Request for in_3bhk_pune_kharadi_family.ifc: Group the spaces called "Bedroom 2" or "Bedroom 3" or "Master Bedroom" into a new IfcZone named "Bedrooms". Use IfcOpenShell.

First a look at what the model holds.

```python
import ifcopenshell

model = ifcopenshell.open("in_3bhk_pune_kharadi_family.ifc")
print(model.schema)
seen = {}
for space in model.by_type("IfcSpace"):
    seen[space.LongName] = seen.get(space.LongName, 0) + 1
for name, count in sorted(seen.items(), key=str):
    print(count, "x", name)
print("zones:", [z.Name for z in model.by_type("IfcZone")][:20])
```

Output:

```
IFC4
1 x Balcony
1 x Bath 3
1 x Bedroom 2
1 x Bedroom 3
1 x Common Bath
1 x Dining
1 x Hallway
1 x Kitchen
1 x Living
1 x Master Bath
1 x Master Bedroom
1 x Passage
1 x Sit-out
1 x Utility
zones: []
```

```python
import ifcopenshell
import ifcopenshell.api.group
import ifcopenshell.api.root

model = ifcopenshell.open("in_3bhk_pune_kharadi_family.ifc")

names = {"Bedroom 2", "Bedroom 3", "Master Bedroom"}
spaces = [s for s in model.by_type("IfcSpace") if s.LongName in names]

zone = ifcopenshell.api.root.create_entity(model, ifc_class="IfcZone", name="Bedrooms")
ifcopenshell.api.group.assign_group(model, products=spaces, group=zone)
print(len(spaces), "spaces in", zone.Name)

model.write("in_3bhk_pune_kharadi_family_updated.ifc")
```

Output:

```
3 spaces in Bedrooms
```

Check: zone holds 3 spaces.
